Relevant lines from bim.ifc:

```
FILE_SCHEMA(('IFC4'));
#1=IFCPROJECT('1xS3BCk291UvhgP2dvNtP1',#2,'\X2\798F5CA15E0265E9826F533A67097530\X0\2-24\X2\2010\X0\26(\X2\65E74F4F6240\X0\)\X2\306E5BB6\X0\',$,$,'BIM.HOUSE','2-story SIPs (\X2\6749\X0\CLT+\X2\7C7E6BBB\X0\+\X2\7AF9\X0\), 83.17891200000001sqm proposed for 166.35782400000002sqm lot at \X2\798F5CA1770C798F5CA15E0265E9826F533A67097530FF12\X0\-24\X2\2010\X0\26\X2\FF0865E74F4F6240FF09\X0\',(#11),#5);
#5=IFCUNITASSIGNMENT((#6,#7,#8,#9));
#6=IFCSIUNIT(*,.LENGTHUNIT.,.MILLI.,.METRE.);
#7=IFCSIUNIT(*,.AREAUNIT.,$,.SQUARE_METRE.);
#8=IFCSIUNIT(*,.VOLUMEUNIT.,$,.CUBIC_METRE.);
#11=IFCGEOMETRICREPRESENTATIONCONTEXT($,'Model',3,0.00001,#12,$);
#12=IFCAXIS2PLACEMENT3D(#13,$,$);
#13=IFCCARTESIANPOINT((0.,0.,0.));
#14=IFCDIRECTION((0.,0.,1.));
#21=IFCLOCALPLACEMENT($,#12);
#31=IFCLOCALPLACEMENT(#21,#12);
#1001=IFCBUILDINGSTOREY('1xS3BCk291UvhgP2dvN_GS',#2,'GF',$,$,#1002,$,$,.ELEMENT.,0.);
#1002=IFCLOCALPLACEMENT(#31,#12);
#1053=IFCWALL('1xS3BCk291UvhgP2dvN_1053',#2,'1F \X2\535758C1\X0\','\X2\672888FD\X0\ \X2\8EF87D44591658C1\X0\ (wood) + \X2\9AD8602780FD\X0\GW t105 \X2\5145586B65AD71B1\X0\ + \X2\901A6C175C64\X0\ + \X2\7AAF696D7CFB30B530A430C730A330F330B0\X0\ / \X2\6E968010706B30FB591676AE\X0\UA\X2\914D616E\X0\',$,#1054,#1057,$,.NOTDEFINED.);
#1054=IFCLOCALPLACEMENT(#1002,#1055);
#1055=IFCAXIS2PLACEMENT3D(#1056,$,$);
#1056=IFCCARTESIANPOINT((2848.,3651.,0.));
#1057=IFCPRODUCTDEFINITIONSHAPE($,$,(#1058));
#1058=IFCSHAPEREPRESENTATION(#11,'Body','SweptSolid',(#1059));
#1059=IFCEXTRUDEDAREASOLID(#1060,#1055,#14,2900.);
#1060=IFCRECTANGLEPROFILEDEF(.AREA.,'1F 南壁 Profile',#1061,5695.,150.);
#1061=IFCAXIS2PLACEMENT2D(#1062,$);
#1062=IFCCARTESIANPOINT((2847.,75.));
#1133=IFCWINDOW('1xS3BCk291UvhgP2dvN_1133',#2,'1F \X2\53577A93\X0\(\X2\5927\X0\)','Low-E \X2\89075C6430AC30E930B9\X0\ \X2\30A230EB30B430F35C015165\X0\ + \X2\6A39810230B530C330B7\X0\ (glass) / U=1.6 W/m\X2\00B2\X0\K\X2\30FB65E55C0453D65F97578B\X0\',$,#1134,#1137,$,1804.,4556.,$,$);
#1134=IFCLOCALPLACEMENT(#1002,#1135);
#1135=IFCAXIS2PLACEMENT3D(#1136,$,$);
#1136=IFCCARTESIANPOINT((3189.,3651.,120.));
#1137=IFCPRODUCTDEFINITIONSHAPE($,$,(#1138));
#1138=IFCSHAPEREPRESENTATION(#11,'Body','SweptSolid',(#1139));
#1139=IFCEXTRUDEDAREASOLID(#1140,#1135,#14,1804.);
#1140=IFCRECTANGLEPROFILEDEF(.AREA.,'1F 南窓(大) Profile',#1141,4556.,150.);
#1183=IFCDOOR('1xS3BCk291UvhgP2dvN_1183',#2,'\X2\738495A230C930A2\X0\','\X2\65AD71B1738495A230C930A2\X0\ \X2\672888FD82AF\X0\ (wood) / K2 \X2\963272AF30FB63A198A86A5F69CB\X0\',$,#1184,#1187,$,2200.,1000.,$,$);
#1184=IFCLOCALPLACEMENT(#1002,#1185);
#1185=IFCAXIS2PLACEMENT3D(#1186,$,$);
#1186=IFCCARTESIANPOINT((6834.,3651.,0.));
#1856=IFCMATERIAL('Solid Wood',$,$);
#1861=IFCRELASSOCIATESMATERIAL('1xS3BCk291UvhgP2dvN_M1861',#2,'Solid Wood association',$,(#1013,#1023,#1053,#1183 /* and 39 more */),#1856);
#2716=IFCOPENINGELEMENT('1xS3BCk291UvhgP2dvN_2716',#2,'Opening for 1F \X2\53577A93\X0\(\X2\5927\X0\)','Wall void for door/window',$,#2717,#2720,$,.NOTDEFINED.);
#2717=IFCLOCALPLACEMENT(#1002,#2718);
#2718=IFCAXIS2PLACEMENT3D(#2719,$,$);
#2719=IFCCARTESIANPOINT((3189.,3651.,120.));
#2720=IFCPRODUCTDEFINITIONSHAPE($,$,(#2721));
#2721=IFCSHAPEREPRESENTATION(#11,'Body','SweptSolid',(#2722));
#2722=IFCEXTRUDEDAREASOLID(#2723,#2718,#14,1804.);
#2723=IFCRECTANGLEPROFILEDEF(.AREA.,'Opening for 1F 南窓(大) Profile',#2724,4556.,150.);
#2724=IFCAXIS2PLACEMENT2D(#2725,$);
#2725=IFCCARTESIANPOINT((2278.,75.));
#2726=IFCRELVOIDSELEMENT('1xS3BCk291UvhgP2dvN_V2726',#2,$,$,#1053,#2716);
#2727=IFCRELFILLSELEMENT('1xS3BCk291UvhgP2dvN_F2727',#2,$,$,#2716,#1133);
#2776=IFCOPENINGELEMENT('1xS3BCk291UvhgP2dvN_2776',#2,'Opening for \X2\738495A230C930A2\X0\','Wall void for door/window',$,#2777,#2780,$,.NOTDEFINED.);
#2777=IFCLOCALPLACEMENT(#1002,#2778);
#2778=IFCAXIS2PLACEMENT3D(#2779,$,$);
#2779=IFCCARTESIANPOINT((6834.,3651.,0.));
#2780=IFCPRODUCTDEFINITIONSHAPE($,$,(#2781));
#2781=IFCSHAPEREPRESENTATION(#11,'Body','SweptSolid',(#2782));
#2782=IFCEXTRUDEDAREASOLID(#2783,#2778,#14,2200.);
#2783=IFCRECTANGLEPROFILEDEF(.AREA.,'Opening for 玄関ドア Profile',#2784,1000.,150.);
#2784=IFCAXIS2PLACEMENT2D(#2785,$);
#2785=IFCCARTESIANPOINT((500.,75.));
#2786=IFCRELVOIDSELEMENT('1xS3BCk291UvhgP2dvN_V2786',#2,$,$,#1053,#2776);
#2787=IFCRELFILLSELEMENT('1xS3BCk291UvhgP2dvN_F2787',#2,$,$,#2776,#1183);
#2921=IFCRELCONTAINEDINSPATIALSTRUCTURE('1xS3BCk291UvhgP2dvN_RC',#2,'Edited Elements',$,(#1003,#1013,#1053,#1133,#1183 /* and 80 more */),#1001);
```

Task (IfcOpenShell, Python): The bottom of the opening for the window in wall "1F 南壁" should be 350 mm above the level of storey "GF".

```python
import numpy as np
import ifcopenshell
import ifcopenshell.api.geometry
import ifcopenshell.geom
import ifcopenshell.util.element
import ifcopenshell.util.placement
import ifcopenshell.util.shape
import ifcopenshell.util.unit

model = ifcopenshell.open("bim.ifc")
unit_scale = ifcopenshell.util.unit.calculate_unit_scale(model)

window = model.by_id(1133)
opening = window.FillsVoids[0].RelatingOpeningElement
storey = ifcopenshell.util.element.get_container(window, ifc_class="IfcBuildingStorey")
level = ifcopenshell.util.placement.get_local_placement(storey.ObjectPlacement)[2, 3]

# The opening's origin need not be at the sill, so measure its lowest point.
shape = ifcopenshell.geom.create_shape(ifcopenshell.geom.settings(), opening)
bottom = ifcopenshell.util.shape.get_shape_bottom_elevation(shape, shape.geometry) / unit_scale
dz = level + 350.0 - bottom

shift = np.array([0.0, 0.0, dz])
# The window is not placed relative to its opening, so move both.
for product in (opening, window):
    matrix = ifcopenshell.util.placement.get_local_placement(product.ObjectPlacement)
    matrix[:3, 3] += shift
    ifcopenshell.api.geometry.edit_object_placement(model, product=product, matrix=matrix, is_si=False)

print(f"moved by {dz * unit_scale:+.3f} m")

model.write("bim-out.ifc")
```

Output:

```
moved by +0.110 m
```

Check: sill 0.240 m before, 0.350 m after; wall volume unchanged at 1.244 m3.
